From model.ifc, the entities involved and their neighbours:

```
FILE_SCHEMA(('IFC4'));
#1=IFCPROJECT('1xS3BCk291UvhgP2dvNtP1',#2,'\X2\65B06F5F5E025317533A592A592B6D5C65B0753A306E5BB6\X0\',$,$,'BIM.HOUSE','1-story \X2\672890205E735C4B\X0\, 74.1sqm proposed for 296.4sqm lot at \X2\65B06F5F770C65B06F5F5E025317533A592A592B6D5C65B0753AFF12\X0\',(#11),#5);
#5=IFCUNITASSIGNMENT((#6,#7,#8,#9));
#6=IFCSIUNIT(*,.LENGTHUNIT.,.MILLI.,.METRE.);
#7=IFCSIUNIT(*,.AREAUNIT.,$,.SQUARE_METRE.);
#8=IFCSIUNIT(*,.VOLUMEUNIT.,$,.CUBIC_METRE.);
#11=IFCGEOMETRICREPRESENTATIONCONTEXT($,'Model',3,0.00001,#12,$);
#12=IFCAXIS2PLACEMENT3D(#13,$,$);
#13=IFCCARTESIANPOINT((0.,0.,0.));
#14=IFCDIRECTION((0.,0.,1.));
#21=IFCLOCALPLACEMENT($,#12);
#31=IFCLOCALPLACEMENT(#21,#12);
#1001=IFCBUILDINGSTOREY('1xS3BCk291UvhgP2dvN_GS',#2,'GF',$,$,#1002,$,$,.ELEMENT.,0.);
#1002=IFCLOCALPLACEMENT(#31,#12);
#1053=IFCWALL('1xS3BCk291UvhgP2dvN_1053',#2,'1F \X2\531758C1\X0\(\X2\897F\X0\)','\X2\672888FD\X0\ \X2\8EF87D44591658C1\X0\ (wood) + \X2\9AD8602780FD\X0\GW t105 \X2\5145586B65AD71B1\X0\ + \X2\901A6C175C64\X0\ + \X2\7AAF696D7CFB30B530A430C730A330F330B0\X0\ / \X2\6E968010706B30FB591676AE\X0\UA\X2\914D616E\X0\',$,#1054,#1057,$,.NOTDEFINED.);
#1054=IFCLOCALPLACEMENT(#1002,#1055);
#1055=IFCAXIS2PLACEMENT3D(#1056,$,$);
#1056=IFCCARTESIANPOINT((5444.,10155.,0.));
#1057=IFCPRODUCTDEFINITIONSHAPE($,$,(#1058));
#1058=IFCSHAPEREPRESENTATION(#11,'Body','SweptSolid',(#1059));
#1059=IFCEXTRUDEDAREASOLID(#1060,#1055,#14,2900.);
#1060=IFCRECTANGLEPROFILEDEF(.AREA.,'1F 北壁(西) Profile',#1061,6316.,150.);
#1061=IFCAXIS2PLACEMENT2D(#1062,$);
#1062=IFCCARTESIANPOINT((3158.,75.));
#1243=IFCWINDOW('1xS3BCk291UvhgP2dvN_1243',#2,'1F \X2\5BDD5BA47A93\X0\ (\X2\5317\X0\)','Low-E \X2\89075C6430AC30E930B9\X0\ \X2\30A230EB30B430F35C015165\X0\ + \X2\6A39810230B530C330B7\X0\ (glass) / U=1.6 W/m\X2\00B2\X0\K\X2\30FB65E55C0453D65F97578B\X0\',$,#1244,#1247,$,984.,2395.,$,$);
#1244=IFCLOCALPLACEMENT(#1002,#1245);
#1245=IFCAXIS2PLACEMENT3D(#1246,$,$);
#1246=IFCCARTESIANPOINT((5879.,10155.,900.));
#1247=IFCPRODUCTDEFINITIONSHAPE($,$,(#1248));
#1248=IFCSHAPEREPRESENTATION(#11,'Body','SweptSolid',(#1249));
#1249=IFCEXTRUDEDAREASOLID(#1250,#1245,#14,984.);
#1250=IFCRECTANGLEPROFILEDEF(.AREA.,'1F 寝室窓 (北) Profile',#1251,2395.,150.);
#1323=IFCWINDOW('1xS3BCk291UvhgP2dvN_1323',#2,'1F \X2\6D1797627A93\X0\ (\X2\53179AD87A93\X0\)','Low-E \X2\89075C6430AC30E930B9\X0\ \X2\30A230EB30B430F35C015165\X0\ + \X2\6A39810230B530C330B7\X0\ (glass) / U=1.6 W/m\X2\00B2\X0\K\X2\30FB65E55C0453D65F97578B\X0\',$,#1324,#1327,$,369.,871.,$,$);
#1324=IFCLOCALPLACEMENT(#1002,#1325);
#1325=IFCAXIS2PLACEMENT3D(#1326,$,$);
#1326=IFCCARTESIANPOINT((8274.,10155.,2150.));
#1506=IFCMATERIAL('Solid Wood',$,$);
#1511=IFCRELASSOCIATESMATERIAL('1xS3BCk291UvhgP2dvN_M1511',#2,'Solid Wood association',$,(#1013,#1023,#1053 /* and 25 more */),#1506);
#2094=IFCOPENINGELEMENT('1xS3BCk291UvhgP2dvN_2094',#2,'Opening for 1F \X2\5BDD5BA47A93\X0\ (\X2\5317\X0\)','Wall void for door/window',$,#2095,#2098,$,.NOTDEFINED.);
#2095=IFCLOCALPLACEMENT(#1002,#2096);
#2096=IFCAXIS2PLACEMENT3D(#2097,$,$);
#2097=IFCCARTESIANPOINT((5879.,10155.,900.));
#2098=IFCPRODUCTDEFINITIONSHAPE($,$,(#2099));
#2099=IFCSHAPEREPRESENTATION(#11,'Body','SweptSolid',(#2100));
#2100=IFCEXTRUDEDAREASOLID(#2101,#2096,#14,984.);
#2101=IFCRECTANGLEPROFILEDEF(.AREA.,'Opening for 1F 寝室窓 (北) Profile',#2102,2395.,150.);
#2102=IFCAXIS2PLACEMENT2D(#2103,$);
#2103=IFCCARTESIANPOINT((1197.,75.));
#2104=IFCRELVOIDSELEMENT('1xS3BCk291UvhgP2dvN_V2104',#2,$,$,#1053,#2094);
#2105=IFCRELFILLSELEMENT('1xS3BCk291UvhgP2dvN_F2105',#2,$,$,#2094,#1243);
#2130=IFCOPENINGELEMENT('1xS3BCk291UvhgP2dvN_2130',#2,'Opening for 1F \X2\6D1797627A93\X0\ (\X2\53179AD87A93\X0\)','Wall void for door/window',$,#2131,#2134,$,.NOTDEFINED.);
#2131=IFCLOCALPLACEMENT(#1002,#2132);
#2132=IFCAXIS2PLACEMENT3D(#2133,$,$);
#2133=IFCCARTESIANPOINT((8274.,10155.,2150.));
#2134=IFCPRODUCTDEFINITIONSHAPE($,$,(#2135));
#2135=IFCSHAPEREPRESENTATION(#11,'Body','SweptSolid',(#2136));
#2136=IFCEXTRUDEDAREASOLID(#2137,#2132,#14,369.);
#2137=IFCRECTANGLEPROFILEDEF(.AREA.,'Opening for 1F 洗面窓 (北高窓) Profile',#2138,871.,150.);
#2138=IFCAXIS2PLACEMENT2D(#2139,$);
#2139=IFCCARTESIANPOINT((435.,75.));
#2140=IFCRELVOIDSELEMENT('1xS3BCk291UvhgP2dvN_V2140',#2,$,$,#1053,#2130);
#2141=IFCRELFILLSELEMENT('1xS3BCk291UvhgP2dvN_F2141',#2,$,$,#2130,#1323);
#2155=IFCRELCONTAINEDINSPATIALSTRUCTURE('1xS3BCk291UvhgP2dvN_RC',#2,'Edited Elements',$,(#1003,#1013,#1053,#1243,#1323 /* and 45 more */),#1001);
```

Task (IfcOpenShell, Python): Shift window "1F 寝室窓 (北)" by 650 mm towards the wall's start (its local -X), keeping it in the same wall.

```python
import ifcopenshell
import ifcopenshell.api.geometry
import ifcopenshell.util.placement
import ifcopenshell.util.unit

model = ifcopenshell.open("model.ifc")
unit_scale = ifcopenshell.util.unit.calculate_unit_scale(model)

window = model.by_guid("1xS3BCk291UvhgP2dvN_1243")
opening = window.FillsVoids[0].RelatingOpeningElement
wall = opening.VoidsElements[0].RelatingBuildingElement

wall_matrix = ifcopenshell.util.placement.get_local_placement(wall.ObjectPlacement)
shift = wall_matrix[:3, 0] * -0.65 / unit_scale
before = ifcopenshell.util.placement.get_local_placement(window.ObjectPlacement)[:3, 3].copy()

# The window is not placed relative to its opening, so move both.
for product in (opening, window):
    matrix = ifcopenshell.util.placement.get_local_placement(product.ObjectPlacement)
    matrix[:3, 3] += shift
    ifcopenshell.api.geometry.edit_object_placement(model, product=product, matrix=matrix, is_si=False)

after = ifcopenshell.util.placement.get_local_placement(window.ObjectPlacement)[:3, 3]
print("window moved by", (after - before).round(3) + 0.0)

model.write("model_updated.ifc")
```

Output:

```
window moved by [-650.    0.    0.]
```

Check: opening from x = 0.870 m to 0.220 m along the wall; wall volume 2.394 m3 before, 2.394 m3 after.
